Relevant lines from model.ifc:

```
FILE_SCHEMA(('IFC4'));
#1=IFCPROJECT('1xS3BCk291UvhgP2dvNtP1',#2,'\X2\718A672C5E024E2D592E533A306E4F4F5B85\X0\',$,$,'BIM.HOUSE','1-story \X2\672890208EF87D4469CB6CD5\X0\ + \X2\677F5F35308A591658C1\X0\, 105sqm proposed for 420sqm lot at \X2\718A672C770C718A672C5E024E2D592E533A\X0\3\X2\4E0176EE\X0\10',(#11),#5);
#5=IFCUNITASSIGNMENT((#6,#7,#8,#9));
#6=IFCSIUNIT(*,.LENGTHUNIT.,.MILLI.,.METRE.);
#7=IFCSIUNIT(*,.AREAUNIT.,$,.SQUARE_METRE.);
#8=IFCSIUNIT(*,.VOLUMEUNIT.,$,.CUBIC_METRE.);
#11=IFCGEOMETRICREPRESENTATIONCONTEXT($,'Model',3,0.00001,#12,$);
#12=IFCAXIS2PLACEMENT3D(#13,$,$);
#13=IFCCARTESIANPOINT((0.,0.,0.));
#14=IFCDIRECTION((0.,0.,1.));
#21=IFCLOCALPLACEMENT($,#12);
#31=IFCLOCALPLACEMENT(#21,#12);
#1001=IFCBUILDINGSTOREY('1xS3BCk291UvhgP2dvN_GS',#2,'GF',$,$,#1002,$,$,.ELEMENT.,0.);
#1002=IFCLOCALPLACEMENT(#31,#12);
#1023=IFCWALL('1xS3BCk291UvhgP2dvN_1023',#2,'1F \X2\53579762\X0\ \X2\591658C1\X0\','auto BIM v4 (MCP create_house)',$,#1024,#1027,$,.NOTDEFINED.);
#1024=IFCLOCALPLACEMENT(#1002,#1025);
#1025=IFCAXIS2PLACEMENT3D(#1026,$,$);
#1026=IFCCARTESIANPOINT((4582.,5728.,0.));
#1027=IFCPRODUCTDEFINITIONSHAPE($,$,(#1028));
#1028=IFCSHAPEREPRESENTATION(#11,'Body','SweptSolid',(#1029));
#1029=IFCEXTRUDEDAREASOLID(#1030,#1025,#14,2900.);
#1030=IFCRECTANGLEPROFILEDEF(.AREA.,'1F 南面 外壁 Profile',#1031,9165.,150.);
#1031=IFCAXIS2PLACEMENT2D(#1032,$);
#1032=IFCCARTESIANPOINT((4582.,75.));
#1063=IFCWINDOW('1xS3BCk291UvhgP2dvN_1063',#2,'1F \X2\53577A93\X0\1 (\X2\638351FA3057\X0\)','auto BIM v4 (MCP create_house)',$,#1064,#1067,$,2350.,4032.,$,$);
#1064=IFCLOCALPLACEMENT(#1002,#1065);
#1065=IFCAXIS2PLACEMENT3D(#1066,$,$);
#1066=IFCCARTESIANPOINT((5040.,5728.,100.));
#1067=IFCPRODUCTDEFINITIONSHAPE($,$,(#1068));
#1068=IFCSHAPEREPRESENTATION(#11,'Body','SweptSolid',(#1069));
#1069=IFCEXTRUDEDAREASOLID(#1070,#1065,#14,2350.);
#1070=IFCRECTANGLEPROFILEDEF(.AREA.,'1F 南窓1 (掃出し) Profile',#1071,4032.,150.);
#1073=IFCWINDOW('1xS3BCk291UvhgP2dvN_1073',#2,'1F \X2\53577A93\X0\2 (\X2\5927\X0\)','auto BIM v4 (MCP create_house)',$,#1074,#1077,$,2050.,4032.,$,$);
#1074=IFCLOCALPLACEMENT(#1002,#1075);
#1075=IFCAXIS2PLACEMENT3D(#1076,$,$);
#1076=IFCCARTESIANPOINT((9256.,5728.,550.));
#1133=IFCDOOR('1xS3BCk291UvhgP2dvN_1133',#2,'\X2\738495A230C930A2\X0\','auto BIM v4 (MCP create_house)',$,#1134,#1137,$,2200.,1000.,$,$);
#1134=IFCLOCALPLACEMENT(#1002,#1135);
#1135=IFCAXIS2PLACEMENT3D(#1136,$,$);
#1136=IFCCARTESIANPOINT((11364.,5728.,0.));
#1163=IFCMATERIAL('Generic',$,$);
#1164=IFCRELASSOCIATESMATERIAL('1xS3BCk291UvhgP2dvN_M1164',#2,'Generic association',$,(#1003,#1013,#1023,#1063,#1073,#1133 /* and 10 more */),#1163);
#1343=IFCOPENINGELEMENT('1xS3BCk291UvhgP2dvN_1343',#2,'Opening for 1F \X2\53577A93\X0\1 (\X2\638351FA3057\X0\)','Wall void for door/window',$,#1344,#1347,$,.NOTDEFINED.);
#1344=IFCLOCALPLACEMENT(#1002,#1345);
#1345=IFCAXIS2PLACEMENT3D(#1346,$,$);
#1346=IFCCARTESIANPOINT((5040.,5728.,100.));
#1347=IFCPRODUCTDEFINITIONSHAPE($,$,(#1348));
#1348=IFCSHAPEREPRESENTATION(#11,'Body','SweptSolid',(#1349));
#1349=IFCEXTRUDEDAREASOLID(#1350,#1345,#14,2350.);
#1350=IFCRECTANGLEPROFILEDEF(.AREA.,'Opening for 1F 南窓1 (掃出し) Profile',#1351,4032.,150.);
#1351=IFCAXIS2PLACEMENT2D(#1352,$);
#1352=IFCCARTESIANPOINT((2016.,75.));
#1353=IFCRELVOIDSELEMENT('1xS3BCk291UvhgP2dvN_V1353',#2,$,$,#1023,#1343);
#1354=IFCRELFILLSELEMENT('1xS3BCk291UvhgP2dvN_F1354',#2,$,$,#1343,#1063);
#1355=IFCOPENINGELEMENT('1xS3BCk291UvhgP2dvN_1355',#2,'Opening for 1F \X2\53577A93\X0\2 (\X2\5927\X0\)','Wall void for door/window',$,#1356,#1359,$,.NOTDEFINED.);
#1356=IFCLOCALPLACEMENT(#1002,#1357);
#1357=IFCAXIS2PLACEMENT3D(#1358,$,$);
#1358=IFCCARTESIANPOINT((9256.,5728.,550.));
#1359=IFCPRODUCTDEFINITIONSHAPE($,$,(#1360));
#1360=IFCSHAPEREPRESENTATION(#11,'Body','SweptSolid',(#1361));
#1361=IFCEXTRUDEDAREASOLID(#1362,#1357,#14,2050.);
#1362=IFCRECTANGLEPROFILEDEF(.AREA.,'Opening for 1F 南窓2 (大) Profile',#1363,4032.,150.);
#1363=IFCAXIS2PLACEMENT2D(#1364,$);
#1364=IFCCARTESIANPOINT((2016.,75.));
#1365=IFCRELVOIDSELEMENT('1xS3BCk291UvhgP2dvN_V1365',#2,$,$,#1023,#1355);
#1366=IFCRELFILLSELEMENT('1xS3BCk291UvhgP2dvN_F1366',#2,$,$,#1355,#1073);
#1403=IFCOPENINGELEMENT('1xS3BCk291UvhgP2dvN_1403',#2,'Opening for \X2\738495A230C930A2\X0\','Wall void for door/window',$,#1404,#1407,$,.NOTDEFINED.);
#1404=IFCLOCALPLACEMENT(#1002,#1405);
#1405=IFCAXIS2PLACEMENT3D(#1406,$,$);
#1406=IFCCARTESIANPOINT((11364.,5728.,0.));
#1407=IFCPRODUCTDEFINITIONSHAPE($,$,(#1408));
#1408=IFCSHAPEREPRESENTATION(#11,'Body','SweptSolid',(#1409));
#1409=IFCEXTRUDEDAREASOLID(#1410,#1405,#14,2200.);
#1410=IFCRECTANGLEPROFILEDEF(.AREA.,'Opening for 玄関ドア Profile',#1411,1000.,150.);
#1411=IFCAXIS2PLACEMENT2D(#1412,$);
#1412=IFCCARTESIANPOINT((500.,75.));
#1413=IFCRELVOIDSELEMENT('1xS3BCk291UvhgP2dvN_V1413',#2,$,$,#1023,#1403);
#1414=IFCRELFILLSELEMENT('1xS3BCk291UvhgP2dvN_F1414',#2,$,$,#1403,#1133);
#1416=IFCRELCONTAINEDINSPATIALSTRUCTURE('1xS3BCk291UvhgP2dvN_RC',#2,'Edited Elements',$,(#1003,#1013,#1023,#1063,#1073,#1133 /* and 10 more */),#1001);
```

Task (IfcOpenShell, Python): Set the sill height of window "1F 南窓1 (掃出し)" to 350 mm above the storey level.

```python
import numpy as np
import ifcopenshell
import ifcopenshell.api.geometry
import ifcopenshell.geom
import ifcopenshell.util.element
import ifcopenshell.util.placement
import ifcopenshell.util.shape
import ifcopenshell.util.unit

model = ifcopenshell.open("model.ifc")
unit_scale = ifcopenshell.util.unit.calculate_unit_scale(model)

window = model.by_guid("1xS3BCk291UvhgP2dvN_1063")
opening = window.FillsVoids[0].RelatingOpeningElement
storey = ifcopenshell.util.element.get_container(window, ifc_class="IfcBuildingStorey")
level = ifcopenshell.util.placement.get_local_placement(storey.ObjectPlacement)[2, 3]

# The opening's origin need not be at the sill, so measure its lowest point.
shape = ifcopenshell.geom.create_shape(ifcopenshell.geom.settings(), opening)
bottom = ifcopenshell.util.shape.get_shape_bottom_elevation(shape, shape.geometry) / unit_scale
dz = level + 0.35 / unit_scale - bottom

shift = np.array([0.0, 0.0, dz])
# The window is not placed relative to its opening, so move both.
for product in (opening, window):
    matrix = ifcopenshell.util.placement.get_local_placement(product.ObjectPlacement)
    matrix[:3, 3] += shift
    ifcopenshell.api.geometry.edit_object_placement(model, product=product, matrix=matrix, is_si=False)

print(f"moved by {dz * unit_scale:+.3f} m")

model.write("model-out.ifc")
```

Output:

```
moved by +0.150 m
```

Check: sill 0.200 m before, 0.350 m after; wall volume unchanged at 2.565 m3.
